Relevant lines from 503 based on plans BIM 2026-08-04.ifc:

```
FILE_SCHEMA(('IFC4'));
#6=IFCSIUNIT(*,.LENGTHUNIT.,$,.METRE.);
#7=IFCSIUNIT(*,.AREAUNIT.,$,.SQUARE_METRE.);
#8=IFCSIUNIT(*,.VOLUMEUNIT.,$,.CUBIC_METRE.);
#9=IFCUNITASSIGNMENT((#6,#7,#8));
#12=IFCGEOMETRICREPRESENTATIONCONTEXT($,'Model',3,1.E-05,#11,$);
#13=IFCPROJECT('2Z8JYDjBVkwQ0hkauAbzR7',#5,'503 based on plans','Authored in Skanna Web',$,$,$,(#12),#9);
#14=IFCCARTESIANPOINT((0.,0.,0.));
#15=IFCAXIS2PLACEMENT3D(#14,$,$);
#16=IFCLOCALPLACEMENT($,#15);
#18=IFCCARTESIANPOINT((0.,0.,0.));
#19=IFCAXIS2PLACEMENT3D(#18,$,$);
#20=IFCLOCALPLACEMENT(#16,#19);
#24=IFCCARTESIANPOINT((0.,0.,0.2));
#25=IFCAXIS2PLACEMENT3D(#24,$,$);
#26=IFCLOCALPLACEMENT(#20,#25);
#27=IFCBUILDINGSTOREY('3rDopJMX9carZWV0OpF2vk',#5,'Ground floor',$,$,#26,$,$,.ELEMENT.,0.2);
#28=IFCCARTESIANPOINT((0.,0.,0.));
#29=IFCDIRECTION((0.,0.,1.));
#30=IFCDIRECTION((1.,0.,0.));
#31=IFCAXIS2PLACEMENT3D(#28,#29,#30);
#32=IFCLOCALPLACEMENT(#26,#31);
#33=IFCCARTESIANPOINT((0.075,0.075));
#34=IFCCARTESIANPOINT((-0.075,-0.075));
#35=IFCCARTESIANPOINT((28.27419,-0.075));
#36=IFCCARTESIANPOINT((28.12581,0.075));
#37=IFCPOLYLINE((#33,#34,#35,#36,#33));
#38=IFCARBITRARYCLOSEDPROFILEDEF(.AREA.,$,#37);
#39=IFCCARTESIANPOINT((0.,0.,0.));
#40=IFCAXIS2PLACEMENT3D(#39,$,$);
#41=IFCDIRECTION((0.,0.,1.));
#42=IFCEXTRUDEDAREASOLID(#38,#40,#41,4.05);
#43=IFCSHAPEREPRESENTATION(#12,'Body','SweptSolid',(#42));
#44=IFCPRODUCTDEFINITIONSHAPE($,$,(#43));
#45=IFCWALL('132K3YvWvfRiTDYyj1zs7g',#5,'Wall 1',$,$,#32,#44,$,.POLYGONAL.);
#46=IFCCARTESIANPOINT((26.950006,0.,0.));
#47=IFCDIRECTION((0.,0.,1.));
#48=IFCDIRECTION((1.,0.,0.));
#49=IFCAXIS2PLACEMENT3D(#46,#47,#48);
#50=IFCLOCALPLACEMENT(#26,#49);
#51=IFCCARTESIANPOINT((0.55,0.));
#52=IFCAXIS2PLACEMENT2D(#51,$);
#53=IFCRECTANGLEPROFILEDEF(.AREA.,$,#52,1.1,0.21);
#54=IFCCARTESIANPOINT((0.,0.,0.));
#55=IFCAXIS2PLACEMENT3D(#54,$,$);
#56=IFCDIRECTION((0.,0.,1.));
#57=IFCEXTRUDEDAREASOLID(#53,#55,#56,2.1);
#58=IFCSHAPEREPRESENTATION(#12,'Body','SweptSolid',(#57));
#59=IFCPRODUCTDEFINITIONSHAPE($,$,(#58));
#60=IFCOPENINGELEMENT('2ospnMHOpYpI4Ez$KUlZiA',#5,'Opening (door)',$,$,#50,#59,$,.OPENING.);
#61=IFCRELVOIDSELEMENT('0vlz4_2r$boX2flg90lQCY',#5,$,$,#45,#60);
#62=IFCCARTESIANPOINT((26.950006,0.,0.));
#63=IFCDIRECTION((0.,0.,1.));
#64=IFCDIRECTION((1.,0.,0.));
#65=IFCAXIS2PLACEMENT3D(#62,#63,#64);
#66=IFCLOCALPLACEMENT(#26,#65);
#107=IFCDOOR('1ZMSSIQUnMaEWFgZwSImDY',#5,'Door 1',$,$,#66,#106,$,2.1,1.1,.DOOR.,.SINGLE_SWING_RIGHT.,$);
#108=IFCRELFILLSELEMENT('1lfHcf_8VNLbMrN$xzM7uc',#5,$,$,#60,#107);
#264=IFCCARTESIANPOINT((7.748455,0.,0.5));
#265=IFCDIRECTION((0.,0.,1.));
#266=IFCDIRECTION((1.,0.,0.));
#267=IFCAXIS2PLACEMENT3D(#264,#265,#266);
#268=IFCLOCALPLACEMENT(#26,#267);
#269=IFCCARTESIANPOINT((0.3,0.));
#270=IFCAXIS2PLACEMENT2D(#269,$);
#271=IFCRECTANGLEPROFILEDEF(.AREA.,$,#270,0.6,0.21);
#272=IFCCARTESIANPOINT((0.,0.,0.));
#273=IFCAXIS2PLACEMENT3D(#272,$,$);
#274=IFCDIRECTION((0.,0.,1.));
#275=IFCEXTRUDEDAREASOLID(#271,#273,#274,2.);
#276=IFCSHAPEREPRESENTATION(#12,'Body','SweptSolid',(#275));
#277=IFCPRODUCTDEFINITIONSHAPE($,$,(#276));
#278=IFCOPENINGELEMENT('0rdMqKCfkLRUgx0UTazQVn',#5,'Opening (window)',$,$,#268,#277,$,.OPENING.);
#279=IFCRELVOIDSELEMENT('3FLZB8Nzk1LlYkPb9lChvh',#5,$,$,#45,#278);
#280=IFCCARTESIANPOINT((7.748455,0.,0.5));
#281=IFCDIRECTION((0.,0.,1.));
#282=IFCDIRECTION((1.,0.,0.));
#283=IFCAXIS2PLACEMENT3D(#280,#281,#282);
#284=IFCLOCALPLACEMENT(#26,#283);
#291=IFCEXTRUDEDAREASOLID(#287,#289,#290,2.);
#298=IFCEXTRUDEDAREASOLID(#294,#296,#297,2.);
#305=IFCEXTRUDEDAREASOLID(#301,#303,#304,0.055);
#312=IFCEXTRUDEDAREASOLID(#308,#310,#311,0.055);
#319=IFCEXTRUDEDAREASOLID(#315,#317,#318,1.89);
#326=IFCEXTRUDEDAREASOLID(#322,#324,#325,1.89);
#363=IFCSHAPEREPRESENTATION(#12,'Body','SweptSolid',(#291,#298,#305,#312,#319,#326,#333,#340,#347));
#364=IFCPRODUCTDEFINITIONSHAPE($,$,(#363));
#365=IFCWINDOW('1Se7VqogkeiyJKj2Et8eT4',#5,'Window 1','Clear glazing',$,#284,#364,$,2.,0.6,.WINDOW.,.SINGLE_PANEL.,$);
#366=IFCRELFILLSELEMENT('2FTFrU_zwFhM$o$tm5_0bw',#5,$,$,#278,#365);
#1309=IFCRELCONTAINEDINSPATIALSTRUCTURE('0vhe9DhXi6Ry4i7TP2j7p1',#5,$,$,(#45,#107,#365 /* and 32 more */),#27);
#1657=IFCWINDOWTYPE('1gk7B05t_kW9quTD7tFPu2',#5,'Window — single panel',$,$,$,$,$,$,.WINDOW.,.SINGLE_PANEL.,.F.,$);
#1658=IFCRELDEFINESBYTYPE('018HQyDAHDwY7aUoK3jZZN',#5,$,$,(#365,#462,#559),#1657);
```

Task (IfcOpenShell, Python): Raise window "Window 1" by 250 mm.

```python
import numpy as np
import ifcopenshell
import ifcopenshell.api.geometry
import ifcopenshell.util.placement
import ifcopenshell.util.unit

model = ifcopenshell.open("503 based on plans BIM 2026-08-04.ifc")
unit_scale = ifcopenshell.util.unit.calculate_unit_scale(model)

window = model.by_guid("1Se7VqogkeiyJKj2Et8eT4")
opening = window.FillsVoids[0].RelatingOpeningElement
dz = 0.25 / unit_scale

shift = np.array([0.0, 0.0, dz])
# The window is not placed relative to its opening, so move both.
for product in (opening, window):
    matrix = ifcopenshell.util.placement.get_local_placement(product.ObjectPlacement)
    matrix[:3, 3] += shift
    ifcopenshell.api.geometry.edit_object_placement(model, product=product, matrix=matrix, is_si=False)

print(f"moved by {dz * unit_scale:+.3f} m")

model.write("503 based on plans BIM 2026-08-04_rev.ifc")
```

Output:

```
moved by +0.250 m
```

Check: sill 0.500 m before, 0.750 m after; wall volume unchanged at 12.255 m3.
